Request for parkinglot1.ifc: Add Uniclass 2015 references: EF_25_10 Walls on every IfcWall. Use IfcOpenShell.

First a look at what the model holds.

```python
import ifcopenshell

model = ifcopenshell.open("parkinglot1.ifc")
print(model.schema)
print("classifications:", [c.Name for c in model.by_type("IfcClassification")])
for ifc_class in ("IfcDoor", "IfcRoof", "IfcStair", "IfcWall", "IfcWindow"):
    print(ifc_class, len(model.by_type(ifc_class)))
```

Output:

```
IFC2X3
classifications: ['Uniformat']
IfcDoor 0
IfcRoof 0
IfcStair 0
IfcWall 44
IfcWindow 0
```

```python
import ifcopenshell
import ifcopenshell.api.classification

model = ifcopenshell.open("parkinglot1.ifc")

# IFC2X3 requires Source and Edition and has no link from the project to the system.
system = model.create_entity("IfcClassification", Source="NBS", Edition="2015", Name="Uniclass 2015")

codes = {
    "IfcWall": ("EF_25_10", "Walls"),
}
for ifc_class, (code, name) in codes.items():
    products = model.by_type(ifc_class)
    ifcopenshell.api.classification.add_reference(
        model, products=products, classification=system, identification=code, name=name
    )
    print(code, len(products))

model.write("parkinglot1_updated.ifc")
```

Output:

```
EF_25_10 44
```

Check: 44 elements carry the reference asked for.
